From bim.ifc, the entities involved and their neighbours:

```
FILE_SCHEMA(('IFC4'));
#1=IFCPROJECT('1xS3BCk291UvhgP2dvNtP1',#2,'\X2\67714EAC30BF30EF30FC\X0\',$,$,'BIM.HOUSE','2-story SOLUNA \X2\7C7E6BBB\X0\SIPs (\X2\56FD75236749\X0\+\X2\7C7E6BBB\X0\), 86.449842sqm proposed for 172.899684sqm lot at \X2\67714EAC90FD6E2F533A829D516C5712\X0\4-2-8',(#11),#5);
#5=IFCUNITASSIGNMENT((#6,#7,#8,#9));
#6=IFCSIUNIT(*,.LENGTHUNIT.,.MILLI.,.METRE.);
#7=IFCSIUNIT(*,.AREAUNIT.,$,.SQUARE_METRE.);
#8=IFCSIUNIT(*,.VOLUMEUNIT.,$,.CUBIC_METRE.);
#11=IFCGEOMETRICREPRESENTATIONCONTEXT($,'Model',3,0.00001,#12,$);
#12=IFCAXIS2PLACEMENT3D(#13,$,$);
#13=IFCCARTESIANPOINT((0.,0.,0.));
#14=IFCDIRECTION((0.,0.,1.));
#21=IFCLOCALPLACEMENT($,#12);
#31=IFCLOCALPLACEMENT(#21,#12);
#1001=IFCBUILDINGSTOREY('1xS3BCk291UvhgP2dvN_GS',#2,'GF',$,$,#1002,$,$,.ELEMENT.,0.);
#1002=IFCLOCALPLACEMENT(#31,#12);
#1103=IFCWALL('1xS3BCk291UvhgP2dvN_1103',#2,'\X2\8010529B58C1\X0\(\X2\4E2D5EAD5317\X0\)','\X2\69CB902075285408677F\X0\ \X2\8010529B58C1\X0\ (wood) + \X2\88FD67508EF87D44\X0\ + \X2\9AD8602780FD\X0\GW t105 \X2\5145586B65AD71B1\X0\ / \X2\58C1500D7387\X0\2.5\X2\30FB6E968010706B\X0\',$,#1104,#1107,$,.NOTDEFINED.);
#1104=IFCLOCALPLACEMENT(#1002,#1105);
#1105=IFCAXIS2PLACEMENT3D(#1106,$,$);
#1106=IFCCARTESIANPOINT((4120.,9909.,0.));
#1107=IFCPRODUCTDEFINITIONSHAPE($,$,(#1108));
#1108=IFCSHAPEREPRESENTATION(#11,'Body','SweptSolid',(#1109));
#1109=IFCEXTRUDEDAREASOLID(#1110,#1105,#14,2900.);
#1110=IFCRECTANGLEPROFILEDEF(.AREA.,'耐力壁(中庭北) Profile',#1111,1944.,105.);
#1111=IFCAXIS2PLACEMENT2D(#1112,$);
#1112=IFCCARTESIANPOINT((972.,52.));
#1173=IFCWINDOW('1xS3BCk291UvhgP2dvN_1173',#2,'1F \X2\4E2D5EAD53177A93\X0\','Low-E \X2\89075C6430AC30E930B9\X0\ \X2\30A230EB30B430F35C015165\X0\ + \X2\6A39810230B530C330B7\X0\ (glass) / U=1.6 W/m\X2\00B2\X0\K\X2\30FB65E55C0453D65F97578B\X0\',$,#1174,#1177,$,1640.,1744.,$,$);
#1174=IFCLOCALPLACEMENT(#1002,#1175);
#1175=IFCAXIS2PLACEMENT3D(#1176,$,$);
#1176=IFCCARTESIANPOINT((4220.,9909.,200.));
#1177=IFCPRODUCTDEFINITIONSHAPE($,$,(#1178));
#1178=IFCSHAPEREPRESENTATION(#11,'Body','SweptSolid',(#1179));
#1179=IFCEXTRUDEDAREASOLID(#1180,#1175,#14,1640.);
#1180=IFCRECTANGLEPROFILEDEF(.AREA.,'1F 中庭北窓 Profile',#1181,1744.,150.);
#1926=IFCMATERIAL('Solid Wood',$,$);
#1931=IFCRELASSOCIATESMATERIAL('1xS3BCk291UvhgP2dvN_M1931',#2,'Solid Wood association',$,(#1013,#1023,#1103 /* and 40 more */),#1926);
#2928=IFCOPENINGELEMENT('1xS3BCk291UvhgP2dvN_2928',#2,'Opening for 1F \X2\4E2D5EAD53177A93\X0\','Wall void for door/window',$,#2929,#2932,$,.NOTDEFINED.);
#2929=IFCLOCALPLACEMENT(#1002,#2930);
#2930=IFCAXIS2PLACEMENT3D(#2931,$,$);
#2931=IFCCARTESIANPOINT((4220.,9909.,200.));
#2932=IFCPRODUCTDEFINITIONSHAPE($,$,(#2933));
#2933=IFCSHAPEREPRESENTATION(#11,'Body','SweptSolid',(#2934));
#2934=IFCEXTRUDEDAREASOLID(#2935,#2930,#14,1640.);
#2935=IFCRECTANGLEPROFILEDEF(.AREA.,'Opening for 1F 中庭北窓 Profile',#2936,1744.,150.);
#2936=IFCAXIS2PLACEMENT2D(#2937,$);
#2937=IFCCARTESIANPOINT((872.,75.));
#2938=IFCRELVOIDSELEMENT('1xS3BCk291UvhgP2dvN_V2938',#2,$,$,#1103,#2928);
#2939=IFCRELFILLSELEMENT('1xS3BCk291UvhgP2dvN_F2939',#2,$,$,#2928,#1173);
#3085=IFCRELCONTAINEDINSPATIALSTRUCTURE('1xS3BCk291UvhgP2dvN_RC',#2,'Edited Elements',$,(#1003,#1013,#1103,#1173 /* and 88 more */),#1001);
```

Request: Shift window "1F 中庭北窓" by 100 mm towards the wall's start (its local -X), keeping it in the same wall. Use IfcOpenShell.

```python
import ifcopenshell
import ifcopenshell.api.geometry
import ifcopenshell.util.placement

model = ifcopenshell.open("bim.ifc")

window = model.by_guid("1xS3BCk291UvhgP2dvN_1173")
opening = window.FillsVoids[0].RelatingOpeningElement
wall = opening.VoidsElements[0].RelatingBuildingElement

wall_matrix = ifcopenshell.util.placement.get_local_placement(wall.ObjectPlacement)
shift = wall_matrix[:3, 0] * -100.0
before = ifcopenshell.util.placement.get_local_placement(window.ObjectPlacement)[:3, 3].copy()

# The window is not placed relative to its opening, so move both.
for product in (opening, window):
    matrix = ifcopenshell.util.placement.get_local_placement(product.ObjectPlacement)
    matrix[:3, 3] += shift
    ifcopenshell.api.geometry.edit_object_placement(model, product=product, matrix=matrix, is_si=False)

after = ifcopenshell.util.placement.get_local_placement(window.ObjectPlacement)[:3, 3]
print("window moved by", (after - before).round(3) + 0.0)

model.write("bim_rev.ifc")
```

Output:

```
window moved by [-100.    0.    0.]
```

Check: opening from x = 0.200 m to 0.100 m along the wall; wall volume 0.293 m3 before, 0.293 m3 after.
